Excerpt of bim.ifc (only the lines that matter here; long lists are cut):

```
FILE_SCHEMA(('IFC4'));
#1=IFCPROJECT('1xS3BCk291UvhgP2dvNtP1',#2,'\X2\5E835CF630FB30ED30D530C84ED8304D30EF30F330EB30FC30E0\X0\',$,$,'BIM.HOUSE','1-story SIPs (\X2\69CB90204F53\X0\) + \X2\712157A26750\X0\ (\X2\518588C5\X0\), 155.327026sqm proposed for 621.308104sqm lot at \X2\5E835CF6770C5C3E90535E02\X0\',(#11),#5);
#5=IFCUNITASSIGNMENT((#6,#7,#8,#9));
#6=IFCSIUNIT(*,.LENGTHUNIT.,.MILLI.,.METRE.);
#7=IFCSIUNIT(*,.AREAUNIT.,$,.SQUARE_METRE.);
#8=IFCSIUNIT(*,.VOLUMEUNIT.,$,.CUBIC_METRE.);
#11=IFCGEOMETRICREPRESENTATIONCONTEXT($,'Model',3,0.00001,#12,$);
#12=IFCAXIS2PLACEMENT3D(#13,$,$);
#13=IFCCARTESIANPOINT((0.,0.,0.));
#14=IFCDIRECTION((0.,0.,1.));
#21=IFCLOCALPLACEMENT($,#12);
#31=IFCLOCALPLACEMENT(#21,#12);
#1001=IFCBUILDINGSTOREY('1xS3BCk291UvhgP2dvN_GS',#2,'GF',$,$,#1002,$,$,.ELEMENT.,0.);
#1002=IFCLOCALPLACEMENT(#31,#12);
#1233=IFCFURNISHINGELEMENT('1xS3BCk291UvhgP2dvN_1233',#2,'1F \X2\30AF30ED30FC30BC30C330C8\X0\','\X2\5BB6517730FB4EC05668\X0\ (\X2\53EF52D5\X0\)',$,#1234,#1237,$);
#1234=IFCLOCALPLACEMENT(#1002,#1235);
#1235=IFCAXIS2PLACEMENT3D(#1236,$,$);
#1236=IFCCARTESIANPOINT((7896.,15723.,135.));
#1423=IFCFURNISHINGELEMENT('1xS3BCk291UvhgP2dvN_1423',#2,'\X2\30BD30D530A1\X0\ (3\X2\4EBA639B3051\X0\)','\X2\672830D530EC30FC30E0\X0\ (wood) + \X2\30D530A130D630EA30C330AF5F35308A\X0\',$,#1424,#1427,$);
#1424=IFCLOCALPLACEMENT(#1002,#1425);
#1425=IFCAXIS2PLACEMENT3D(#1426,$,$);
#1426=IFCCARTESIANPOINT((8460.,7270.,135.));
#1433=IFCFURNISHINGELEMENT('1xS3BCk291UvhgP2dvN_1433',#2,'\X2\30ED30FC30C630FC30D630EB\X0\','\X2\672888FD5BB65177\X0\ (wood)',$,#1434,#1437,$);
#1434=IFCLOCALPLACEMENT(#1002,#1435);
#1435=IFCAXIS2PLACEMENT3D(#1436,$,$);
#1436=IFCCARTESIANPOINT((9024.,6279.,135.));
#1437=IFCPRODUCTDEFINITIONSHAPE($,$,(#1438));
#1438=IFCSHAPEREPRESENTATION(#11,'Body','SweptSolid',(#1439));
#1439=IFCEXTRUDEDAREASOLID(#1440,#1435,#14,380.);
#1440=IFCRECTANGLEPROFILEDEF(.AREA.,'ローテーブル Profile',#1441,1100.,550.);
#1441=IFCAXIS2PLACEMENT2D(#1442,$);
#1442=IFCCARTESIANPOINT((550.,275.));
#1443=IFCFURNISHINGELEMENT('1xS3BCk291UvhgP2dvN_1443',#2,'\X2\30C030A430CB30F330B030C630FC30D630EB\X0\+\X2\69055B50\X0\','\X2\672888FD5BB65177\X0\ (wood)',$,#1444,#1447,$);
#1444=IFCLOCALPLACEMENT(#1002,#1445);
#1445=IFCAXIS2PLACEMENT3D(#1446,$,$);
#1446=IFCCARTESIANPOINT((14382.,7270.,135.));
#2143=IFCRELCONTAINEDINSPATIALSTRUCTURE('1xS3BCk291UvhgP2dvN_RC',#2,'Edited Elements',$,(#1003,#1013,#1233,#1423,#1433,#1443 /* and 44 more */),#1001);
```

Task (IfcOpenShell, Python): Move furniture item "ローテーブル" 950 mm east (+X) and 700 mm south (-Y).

```python
import ifcopenshell
import ifcopenshell.api.geometry
import ifcopenshell.util.placement

model = ifcopenshell.open("bim.ifc")

item = model.by_guid("1xS3BCk291UvhgP2dvN_1433")
matrix = ifcopenshell.util.placement.get_local_placement(item.ObjectPlacement)
matrix[0, 3] += 950.0
matrix[1, 3] -= 700.0
ifcopenshell.api.geometry.edit_object_placement(model, product=item, matrix=matrix, is_si=False)

print(ifcopenshell.util.placement.get_local_placement(item.ObjectPlacement).round(3) + 0.0)

model.write("bim_updated.ifc")
```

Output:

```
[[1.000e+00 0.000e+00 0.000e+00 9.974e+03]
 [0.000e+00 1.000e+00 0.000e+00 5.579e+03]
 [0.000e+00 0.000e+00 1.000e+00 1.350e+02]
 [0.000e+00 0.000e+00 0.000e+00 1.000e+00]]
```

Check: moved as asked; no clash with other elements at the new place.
